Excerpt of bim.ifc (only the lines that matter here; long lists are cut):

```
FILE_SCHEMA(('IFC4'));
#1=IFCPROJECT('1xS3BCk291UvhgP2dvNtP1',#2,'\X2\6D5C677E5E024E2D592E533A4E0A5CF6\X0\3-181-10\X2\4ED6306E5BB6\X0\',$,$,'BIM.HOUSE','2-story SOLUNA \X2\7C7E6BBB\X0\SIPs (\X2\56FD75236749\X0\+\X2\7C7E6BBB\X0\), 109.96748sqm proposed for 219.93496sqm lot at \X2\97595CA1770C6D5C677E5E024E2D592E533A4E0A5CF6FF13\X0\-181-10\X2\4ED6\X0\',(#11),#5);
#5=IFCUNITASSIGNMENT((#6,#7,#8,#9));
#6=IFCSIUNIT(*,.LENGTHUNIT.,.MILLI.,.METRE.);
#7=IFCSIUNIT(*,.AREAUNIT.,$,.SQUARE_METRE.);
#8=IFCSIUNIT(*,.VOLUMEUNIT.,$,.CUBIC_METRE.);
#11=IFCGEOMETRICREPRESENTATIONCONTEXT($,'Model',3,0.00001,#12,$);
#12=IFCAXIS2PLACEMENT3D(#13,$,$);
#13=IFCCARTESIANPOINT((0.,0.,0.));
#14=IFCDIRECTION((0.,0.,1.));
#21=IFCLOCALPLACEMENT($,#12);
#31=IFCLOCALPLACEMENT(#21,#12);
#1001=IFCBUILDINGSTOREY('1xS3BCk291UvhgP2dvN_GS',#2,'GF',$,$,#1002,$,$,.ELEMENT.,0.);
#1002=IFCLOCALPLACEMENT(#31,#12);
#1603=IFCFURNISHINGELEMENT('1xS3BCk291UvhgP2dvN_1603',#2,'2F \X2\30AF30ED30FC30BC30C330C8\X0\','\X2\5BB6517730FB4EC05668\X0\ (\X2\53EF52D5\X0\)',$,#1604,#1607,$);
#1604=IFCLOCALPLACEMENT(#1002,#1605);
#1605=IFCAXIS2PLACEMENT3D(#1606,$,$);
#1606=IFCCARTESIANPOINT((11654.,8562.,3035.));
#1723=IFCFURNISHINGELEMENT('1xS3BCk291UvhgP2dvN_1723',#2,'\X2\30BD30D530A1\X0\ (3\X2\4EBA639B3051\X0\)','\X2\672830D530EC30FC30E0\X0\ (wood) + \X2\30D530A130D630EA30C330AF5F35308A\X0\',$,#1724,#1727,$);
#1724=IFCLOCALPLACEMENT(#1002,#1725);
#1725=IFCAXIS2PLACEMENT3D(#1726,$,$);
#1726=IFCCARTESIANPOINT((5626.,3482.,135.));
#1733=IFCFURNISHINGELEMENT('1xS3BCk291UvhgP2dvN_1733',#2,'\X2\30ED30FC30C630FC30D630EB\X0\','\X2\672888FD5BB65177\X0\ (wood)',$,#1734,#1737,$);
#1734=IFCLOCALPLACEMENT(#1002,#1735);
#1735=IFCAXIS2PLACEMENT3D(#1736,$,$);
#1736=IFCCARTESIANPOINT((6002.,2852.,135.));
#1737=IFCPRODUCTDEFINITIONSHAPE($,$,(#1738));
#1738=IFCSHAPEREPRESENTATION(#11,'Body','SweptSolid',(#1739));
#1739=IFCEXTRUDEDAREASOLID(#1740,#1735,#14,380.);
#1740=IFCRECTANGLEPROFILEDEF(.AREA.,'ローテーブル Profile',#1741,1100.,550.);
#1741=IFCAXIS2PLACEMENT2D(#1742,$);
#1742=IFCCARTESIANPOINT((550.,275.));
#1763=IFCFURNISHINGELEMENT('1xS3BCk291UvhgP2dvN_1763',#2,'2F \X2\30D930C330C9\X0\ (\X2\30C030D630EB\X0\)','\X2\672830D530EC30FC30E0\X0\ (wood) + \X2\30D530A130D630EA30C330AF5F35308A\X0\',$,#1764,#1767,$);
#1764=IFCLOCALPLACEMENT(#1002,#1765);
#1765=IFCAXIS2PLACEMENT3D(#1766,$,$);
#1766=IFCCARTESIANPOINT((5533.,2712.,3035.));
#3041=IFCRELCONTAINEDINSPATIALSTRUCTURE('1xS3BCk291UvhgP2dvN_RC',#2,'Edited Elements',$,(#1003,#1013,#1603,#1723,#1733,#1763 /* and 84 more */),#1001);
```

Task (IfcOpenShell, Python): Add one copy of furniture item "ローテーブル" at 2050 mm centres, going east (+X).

```python
import numpy as np
import ifcopenshell
import ifcopenshell.api.geometry
import ifcopenshell.api.root
import ifcopenshell.util.element
import ifcopenshell.util.placement
import ifcopenshell.util.unit

model = ifcopenshell.open("bim.ifc")
unit_scale = ifcopenshell.util.unit.calculate_unit_scale(model)


def reuse_history(source, copy):
    """copy_class also copies each property set's owner history, people and application; keep the originals."""
    for rel in copy.IsDefinedBy:
        if rel.is_a("IfcRelDefinesByProperties") and (history := rel.RelatingPropertyDefinition.OwnerHistory):
            rel.RelatingPropertyDefinition.OwnerHistory = source.OwnerHistory
            ifcopenshell.util.element.remove_deep2(model, history)


source = model.by_guid("1xS3BCk291UvhgP2dvN_1733")
base = ifcopenshell.util.placement.get_local_placement(source.ObjectPlacement)
step = np.array([1.0, 0.0, 0.0]) * 2.05 / unit_scale

for i in range(1, 2):
    copy = ifcopenshell.api.root.copy_class(model, product=source)
    copy.Representation = ifcopenshell.util.element.copy_deep(
        model, source.Representation, exclude=["IfcGeometricRepresentationContext", "IfcRepresentationMap"]
    )
    reuse_history(source, copy)
    matrix = base.copy()
    matrix[:3, 3] += i * step
    print("added at", matrix[:3, 3].round(3) + 0.0)
    ifcopenshell.api.geometry.edit_object_placement(model, product=copy, matrix=matrix, is_si=False)

model.write("bim_v2.ifc")
```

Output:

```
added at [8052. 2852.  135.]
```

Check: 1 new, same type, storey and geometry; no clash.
